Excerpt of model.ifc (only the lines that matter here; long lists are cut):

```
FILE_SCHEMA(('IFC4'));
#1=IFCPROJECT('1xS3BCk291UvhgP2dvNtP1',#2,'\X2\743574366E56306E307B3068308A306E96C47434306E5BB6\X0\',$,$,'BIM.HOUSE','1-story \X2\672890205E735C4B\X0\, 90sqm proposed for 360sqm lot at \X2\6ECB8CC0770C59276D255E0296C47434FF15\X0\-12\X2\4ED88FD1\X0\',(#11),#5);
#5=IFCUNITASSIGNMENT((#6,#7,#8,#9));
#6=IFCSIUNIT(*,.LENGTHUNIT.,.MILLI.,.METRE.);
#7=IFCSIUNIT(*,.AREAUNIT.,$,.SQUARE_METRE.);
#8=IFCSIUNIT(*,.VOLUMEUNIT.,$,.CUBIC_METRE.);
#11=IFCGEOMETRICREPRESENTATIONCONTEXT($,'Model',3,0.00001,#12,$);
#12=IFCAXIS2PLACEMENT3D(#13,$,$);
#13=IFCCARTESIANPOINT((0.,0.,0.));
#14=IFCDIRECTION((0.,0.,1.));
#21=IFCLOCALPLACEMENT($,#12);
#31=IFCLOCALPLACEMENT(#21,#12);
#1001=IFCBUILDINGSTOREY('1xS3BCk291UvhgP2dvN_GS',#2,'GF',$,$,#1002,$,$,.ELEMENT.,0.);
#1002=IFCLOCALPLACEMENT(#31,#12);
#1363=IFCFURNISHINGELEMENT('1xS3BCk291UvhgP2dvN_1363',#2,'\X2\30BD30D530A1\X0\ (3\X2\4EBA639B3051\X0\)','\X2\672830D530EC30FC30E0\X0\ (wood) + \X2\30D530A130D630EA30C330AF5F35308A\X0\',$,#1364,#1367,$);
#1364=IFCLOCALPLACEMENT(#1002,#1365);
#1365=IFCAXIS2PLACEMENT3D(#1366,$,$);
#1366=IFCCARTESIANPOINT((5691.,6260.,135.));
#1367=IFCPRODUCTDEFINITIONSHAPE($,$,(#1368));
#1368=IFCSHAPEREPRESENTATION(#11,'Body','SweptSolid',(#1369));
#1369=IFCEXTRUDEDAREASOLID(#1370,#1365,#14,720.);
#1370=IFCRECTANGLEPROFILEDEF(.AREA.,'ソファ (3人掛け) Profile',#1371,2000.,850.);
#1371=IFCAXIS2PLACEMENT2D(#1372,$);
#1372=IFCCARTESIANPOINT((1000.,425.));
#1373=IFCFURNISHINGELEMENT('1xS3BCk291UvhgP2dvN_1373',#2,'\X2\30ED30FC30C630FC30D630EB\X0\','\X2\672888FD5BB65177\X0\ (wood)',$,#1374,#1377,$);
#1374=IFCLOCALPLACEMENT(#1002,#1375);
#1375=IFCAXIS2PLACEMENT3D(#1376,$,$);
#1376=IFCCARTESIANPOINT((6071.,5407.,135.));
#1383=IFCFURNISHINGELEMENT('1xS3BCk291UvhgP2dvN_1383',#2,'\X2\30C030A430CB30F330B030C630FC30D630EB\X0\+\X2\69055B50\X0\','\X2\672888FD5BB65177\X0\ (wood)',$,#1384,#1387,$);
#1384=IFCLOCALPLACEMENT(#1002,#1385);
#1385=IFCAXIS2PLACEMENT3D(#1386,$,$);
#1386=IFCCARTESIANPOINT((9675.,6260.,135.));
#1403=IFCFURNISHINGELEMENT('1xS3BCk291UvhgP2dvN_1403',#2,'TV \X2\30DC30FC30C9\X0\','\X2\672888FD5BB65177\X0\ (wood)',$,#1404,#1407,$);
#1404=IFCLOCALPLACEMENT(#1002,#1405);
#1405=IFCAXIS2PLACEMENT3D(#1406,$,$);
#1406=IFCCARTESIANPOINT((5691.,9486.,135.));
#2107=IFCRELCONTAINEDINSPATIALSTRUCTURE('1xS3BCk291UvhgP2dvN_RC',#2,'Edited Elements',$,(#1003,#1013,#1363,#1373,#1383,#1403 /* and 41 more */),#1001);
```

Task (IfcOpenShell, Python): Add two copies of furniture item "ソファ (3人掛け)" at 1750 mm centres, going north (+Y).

```python
import numpy as np
import ifcopenshell
import ifcopenshell.api.geometry
import ifcopenshell.api.root
import ifcopenshell.util.element
import ifcopenshell.util.placement

model = ifcopenshell.open("model.ifc")


def reuse_history(source, copy):
    """copy_class also copies each property set's owner history, people and application; keep the originals."""
    for rel in copy.IsDefinedBy:
        if rel.is_a("IfcRelDefinesByProperties") and (history := rel.RelatingPropertyDefinition.OwnerHistory):
            rel.RelatingPropertyDefinition.OwnerHistory = source.OwnerHistory
            ifcopenshell.util.element.remove_deep2(model, history)


source = model.by_id(1363)
base = ifcopenshell.util.placement.get_local_placement(source.ObjectPlacement)
step = np.array([0.0, 1.0, 0.0]) * 1750.0

for i in range(1, 3):
    copy = ifcopenshell.api.root.copy_class(model, product=source)
    copy.Representation = ifcopenshell.util.element.copy_deep(
        model, source.Representation, exclude=["IfcGeometricRepresentationContext", "IfcRepresentationMap"]
    )
    reuse_history(source, copy)
    matrix = base.copy()
    matrix[:3, 3] += i * step
    print("added at", matrix[:3, 3].round(3) + 0.0)
    ifcopenshell.api.geometry.edit_object_placement(model, product=copy, matrix=matrix, is_si=False)

model.write("model_edited.ifc")
```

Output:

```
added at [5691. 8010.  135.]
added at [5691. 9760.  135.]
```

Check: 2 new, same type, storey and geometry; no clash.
